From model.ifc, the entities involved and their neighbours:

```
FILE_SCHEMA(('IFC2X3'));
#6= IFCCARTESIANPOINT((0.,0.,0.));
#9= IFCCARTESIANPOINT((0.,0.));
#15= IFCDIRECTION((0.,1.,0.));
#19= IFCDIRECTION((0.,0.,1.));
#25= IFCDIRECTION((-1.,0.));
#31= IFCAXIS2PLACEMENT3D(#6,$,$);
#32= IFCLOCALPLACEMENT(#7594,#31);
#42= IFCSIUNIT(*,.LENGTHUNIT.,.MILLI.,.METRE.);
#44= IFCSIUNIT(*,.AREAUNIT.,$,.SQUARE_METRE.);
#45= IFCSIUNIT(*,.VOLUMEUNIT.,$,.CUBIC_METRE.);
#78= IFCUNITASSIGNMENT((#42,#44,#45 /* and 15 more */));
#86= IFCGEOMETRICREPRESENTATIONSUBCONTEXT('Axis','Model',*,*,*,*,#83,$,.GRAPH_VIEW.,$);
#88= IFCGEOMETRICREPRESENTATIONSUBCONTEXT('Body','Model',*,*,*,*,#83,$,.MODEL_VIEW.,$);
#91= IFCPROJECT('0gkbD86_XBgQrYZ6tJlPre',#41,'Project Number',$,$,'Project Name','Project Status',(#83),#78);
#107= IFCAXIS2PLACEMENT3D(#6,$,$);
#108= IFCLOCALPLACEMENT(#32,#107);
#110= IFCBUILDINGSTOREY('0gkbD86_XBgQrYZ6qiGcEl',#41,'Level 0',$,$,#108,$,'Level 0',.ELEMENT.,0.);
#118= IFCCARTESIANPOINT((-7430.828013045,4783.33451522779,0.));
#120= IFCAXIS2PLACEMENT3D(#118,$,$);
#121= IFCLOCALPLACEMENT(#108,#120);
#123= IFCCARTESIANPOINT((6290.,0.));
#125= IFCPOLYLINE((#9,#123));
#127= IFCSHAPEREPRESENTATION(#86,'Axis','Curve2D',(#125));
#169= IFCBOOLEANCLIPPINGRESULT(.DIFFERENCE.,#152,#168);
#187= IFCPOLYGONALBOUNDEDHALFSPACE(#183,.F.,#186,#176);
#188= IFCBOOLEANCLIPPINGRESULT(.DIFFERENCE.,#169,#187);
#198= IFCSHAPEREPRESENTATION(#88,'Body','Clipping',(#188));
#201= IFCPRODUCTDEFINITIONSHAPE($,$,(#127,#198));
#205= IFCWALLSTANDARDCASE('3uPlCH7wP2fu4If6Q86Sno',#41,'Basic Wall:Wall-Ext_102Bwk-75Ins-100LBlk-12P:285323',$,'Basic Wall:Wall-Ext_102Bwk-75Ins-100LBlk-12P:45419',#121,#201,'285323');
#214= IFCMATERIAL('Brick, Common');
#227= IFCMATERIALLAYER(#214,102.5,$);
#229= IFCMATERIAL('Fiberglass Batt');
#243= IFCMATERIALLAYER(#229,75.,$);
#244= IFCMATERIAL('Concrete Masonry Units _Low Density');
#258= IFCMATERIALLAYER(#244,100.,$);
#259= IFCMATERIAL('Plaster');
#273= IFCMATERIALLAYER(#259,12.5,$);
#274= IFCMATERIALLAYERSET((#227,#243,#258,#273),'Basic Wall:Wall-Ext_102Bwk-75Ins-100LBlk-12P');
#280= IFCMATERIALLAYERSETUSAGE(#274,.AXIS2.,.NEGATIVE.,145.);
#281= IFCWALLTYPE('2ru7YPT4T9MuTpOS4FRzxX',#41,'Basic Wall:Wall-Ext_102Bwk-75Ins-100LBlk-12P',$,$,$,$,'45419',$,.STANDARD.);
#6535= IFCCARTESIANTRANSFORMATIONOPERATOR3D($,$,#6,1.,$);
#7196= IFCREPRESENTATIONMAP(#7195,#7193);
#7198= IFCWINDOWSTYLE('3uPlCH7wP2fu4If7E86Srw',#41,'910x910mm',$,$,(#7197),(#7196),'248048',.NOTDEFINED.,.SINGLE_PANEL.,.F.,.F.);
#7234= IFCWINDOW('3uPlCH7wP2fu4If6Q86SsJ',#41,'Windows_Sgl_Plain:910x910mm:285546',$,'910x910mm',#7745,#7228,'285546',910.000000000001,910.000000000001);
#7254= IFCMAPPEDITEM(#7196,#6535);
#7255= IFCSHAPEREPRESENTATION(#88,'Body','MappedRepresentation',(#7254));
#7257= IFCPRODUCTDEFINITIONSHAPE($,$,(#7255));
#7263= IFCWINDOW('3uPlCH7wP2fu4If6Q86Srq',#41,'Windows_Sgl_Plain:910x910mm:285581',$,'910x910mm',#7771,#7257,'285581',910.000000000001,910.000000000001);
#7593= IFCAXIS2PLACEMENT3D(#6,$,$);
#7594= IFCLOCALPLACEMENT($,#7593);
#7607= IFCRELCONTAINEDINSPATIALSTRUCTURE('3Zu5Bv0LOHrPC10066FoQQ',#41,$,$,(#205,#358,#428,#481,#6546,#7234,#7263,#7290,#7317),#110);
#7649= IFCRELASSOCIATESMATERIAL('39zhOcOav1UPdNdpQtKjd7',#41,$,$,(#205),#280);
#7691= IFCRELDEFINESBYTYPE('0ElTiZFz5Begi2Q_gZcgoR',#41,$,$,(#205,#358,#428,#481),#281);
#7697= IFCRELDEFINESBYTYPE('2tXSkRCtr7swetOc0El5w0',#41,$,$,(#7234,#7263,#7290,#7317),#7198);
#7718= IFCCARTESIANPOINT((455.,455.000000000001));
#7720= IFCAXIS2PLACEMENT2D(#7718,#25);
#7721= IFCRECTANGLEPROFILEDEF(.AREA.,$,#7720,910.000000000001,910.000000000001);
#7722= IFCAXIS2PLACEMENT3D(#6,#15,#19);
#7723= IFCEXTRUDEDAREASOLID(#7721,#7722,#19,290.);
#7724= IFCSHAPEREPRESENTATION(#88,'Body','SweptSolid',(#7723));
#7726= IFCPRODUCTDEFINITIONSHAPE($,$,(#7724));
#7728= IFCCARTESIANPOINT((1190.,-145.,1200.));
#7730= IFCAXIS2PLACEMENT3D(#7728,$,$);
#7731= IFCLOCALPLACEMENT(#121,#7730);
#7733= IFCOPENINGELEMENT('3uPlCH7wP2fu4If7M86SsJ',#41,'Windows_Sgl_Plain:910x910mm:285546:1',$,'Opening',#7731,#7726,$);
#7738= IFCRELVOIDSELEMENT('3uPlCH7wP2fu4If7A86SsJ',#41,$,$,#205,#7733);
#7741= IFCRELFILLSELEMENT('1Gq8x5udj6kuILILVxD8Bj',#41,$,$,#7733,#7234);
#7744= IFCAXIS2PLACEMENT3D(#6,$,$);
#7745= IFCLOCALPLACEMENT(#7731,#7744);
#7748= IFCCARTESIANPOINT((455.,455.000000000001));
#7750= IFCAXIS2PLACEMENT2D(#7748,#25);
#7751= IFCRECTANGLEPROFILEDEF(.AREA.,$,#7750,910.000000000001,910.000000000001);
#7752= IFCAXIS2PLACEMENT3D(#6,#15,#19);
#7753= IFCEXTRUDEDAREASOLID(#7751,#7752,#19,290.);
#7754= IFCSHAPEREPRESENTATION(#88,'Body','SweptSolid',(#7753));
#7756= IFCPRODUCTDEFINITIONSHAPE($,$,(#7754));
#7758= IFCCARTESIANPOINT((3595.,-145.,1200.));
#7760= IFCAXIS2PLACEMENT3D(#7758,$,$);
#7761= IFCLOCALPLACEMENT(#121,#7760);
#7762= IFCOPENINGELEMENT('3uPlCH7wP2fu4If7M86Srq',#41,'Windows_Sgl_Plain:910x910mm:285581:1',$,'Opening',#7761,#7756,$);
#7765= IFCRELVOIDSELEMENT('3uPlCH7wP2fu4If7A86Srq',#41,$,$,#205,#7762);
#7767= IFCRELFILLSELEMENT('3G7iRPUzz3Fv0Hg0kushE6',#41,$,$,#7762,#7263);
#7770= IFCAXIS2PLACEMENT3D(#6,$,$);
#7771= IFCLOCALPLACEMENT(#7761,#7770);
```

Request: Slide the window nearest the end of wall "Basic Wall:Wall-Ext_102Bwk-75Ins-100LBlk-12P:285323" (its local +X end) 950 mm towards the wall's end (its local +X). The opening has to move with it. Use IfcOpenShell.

```python
import ifcopenshell
import ifcopenshell.api.geometry
import ifcopenshell.util.placement

model = ifcopenshell.open("model.ifc")

window = model.by_guid("3uPlCH7wP2fu4If6Q86Srq")
opening = window.FillsVoids[0].RelatingOpeningElement
wall = opening.VoidsElements[0].RelatingBuildingElement

wall_matrix = ifcopenshell.util.placement.get_local_placement(wall.ObjectPlacement)
shift = wall_matrix[:3, 0] * 950.0
before = ifcopenshell.util.placement.get_local_placement(window.ObjectPlacement)[:3, 3].copy()

# The window is placed relative to its opening, so it follows when the opening moves.
matrix = ifcopenshell.util.placement.get_local_placement(opening.ObjectPlacement)
matrix[:3, 3] += shift
ifcopenshell.api.geometry.edit_object_placement(
    model, product=opening, matrix=matrix, is_si=False, should_transform_children=True
)

after = ifcopenshell.util.placement.get_local_placement(window.ObjectPlacement)[:3, 3]
print("window moved by", (after - before).round(3) + 0.0)

model.write("model_v2.ifc")
```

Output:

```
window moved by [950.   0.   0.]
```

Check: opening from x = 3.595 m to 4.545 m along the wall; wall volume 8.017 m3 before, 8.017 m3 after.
